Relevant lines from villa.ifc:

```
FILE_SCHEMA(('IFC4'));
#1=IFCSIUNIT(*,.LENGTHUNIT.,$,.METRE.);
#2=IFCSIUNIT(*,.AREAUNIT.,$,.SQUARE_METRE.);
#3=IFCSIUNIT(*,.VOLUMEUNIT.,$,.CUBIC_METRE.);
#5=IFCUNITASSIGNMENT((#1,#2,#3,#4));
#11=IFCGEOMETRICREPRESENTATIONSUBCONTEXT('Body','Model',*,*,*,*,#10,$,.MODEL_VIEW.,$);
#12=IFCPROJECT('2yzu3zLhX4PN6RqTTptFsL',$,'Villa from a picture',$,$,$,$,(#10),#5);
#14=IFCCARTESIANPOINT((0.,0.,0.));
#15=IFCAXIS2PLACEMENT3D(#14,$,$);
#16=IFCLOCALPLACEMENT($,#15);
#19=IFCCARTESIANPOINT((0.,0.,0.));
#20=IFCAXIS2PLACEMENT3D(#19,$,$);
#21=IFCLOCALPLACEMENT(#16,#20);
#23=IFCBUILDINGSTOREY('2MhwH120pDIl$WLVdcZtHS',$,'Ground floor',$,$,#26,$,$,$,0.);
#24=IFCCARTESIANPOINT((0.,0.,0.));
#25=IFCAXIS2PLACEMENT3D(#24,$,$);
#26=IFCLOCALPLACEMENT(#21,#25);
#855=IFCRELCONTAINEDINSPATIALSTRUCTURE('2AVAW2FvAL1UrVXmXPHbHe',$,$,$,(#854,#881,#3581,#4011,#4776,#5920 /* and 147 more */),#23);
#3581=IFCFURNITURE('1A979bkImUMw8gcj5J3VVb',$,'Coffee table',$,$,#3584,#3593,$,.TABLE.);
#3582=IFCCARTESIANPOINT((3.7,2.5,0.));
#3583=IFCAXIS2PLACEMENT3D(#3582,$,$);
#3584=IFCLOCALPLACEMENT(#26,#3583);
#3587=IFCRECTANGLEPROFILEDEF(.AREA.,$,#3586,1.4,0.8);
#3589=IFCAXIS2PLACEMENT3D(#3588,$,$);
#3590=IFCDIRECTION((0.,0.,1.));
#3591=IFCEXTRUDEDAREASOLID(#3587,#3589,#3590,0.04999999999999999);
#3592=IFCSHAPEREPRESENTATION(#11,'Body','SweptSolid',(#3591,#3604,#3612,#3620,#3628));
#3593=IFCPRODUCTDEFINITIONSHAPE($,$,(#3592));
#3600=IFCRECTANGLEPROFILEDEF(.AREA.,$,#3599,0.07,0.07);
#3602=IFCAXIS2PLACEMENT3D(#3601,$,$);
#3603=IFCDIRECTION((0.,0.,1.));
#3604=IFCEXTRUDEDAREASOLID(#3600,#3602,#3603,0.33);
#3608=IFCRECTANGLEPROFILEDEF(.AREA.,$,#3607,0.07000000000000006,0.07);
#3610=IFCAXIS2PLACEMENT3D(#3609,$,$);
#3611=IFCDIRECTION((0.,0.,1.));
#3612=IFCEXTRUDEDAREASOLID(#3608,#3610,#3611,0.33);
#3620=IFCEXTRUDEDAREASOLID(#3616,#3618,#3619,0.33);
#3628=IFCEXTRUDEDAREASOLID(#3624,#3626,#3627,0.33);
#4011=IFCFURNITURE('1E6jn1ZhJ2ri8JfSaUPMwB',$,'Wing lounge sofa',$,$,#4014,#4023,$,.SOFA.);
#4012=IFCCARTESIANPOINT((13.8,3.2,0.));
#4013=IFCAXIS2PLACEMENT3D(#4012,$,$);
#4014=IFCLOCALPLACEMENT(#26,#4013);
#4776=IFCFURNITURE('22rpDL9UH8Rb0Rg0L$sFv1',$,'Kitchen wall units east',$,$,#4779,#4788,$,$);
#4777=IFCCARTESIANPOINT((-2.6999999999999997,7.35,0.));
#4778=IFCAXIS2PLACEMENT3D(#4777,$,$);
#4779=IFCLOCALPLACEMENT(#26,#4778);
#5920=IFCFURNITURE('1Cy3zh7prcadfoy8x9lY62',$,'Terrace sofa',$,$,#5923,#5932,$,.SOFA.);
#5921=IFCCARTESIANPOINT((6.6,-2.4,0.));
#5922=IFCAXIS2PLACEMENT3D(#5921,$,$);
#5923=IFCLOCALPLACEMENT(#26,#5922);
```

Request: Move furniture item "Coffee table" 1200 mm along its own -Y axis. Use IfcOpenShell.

```python
import ifcopenshell
import ifcopenshell.api.geometry
import ifcopenshell.util.placement

model = ifcopenshell.open("villa.ifc")

item = model.by_guid("1A979bkImUMw8gcj5J3VVb")
matrix = ifcopenshell.util.placement.get_local_placement(item.ObjectPlacement)
matrix[:3, 3] -= matrix[:3, 1] * 1.2
ifcopenshell.api.geometry.edit_object_placement(model, product=item, matrix=matrix, is_si=False)

print(ifcopenshell.util.placement.get_local_placement(item.ObjectPlacement).round(3) + 0.0)

model.write("villa_v2.ifc")
```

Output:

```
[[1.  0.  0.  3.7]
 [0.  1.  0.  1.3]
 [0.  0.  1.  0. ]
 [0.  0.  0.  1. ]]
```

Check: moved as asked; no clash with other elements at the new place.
